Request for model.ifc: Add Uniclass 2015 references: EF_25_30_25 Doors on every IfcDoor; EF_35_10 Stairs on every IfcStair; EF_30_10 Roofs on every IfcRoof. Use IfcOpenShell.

First a look at what the model holds.

```python
import ifcopenshell

model = ifcopenshell.open("model.ifc")
print(model.schema)
print("classifications:", [c.Name for c in model.by_type("IfcClassification")])
for ifc_class in ("IfcDoor", "IfcRoof", "IfcStair", "IfcWall", "IfcWindow"):
    print(ifc_class, len(model.by_type(ifc_class)))
```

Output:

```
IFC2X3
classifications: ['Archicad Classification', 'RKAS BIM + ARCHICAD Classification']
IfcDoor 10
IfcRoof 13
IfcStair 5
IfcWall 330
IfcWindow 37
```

```python
import ifcopenshell
import ifcopenshell.api.classification

model = ifcopenshell.open("model.ifc")

# IFC2X3 requires Source and Edition and has no link from the project to the system.
system = model.create_entity("IfcClassification", Source="NBS", Edition="2015", Name="Uniclass 2015")

codes = {
    "IfcDoor": ("EF_25_30_25", "Doors"),
    "IfcStair": ("EF_35_10", "Stairs"),
    "IfcRoof": ("EF_30_10", "Roofs"),
}
for ifc_class, (code, name) in codes.items():
    products = model.by_type(ifc_class)
    ifcopenshell.api.classification.add_reference(
        model, products=products, classification=system, identification=code, name=name
    )
    print(code, len(products))

model.write("model-out.ifc")
```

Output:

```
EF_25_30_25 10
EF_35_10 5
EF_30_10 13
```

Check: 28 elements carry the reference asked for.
